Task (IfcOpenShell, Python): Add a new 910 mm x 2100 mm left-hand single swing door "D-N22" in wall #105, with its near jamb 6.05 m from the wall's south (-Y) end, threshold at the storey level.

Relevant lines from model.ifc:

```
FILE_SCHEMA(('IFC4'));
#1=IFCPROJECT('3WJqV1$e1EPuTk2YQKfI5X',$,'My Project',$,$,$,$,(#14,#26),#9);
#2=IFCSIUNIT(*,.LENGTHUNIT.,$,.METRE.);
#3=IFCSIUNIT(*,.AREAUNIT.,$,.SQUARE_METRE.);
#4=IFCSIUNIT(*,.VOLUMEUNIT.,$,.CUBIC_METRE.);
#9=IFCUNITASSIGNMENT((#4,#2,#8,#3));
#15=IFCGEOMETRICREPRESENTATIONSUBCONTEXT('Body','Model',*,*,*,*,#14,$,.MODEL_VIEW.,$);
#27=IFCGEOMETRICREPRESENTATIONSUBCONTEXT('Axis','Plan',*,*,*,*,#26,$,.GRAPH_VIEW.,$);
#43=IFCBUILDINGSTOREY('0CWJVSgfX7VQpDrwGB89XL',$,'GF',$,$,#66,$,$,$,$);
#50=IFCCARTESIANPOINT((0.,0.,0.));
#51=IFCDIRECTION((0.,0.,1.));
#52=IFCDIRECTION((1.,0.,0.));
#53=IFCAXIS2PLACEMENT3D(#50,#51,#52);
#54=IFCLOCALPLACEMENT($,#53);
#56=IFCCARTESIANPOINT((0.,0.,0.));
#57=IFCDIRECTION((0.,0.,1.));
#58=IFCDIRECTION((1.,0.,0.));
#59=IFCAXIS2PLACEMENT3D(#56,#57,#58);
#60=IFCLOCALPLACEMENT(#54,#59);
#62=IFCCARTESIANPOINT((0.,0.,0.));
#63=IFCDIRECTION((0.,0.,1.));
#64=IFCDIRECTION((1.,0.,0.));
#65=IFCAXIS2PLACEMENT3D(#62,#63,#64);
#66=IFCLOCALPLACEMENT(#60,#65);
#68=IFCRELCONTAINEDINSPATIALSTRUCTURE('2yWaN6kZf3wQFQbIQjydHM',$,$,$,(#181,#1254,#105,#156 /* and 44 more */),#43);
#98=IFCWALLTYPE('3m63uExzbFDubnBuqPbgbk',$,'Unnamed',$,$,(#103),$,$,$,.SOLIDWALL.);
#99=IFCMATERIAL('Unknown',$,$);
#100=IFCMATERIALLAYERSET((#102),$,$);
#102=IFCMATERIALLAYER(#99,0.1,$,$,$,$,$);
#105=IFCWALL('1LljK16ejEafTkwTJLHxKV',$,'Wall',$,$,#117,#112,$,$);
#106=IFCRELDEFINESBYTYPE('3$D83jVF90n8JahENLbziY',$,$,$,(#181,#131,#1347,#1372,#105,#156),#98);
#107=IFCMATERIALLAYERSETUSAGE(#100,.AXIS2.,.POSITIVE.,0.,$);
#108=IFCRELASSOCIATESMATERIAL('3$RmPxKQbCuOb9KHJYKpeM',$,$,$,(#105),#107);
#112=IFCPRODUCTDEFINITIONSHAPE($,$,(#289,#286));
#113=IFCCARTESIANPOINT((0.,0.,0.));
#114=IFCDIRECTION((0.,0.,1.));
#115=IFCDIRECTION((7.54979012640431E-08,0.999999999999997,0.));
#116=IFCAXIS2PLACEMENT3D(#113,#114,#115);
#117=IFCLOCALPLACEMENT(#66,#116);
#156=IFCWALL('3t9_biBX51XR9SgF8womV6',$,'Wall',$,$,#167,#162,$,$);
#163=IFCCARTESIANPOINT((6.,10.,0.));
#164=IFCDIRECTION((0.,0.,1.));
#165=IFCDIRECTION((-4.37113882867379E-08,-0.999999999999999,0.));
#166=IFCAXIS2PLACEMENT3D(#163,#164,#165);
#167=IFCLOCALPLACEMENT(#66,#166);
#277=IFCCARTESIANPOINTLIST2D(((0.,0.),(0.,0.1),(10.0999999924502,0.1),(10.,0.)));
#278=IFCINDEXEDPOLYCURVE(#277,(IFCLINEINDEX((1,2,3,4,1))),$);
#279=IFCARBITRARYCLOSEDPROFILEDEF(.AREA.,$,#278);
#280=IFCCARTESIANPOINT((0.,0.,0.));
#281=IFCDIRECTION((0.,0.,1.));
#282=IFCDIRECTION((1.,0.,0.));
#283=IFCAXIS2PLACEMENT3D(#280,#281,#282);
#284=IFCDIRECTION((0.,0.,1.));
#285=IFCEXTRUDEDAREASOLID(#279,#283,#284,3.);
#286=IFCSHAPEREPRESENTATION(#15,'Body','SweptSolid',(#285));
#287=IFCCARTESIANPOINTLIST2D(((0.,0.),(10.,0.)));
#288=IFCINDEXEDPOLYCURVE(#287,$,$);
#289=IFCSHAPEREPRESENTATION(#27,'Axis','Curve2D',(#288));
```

```python
import numpy as np
import ifcopenshell
import ifcopenshell.api.feature
import ifcopenshell.api.geometry
import ifcopenshell.api.root
import ifcopenshell.api.spatial
import ifcopenshell.geom
import ifcopenshell.util.element
import ifcopenshell.util.placement
import ifcopenshell.util.representation
import ifcopenshell.util.shape
import ifcopenshell.util.unit

model = ifcopenshell.open("model.ifc")
unit_scale = ifcopenshell.util.unit.calculate_unit_scale(model)
settings = ifcopenshell.geom.settings()


def volume(element):
    """Net volume in cubic metres, openings subtracted."""
    shape = ifcopenshell.geom.create_shape(settings, element)
    return ifcopenshell.util.shape.get_volume(shape.geometry)


wall = model.by_guid("1LljK16ejEafTkwTJLHxKV")
storey = ifcopenshell.util.element.get_container(wall, ifc_class="IfcBuildingStorey")
context = ifcopenshell.util.representation.get_context(model, "Model", "Body", "MODEL_VIEW")
before = volume(wall)

width, height, from_end, sill = 0.91, 2.1, 6.05, 0.0  # metres

# The wall runs along its own X axis, and the end named is its -X end.
wall_shape = ifcopenshell.geom.create_shape(settings, wall)
x, y, z = ifcopenshell.util.shape.get_vertices(wall_shape.geometry).T
start = x.min() + from_end
face, thickness = float(y.min()), float(y.max() - y.min())
wall_matrix = ifcopenshell.util.placement.get_local_placement(wall.ObjectPlacement)
level = ifcopenshell.util.placement.get_local_placement(storey.ObjectPlacement)[2, 3]


def in_wall(x, y):
    """Placement at x, y metres in the wall's axes, at sill height."""
    matrix = wall_matrix.copy()
    matrix[:, 3] = wall_matrix @ np.array([x / unit_scale, y / unit_scale, 0.0, 1.0])
    matrix[2, 3] = level + sill / unit_scale
    return matrix


# Opening: a box that overshoots both wall faces by 50 mm.
opening = ifcopenshell.api.root.create_entity(model, ifc_class="IfcOpeningElement", predefined_type="OPENING")
box = ifcopenshell.api.geometry.add_wall_representation(
    model, context=context, length=width, height=height, thickness=thickness + 0.1
)
ifcopenshell.api.geometry.assign_representation(model, product=opening, representation=box)
ifcopenshell.api.geometry.edit_object_placement(model, product=opening, matrix=in_wall(start, face - 0.05), is_si=False)
ifcopenshell.api.feature.add_feature(model, feature=opening, element=wall)

door = ifcopenshell.api.root.create_entity(model, ifc_class="IfcDoor", name="D-N22", predefined_type="DOOR")
door.OverallWidth, door.OverallHeight = width / unit_scale, height / unit_scale
door.OperationType = "SINGLE_SWING_LEFT"
body = ifcopenshell.api.geometry.add_door_representation(
    model,
    context=context,
    overall_width=door.OverallWidth,
    overall_height=door.OverallHeight,
    operation_type="SINGLE_SWING_LEFT",
    lining_properties={"LiningDepth": thickness / unit_scale, "ThresholdDepth": thickness / unit_scale},
)
ifcopenshell.api.geometry.assign_representation(model, product=door, representation=body)
ifcopenshell.api.spatial.assign_container(model, products=[door], relating_structure=storey)
ifcopenshell.api.feature.add_filling(model, opening=opening, element=door)

# The lining spans the wall, so the door starts at the wall face.
ifcopenshell.api.geometry.edit_object_placement(model, product=door, matrix=in_wall(start, face), is_si=False)

after = volume(wall)

print(f"wall volume {before:.3f} -> {after:.3f} m3")

model.write("model_edited.ifc")
```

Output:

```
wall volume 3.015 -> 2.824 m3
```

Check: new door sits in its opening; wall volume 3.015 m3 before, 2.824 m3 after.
